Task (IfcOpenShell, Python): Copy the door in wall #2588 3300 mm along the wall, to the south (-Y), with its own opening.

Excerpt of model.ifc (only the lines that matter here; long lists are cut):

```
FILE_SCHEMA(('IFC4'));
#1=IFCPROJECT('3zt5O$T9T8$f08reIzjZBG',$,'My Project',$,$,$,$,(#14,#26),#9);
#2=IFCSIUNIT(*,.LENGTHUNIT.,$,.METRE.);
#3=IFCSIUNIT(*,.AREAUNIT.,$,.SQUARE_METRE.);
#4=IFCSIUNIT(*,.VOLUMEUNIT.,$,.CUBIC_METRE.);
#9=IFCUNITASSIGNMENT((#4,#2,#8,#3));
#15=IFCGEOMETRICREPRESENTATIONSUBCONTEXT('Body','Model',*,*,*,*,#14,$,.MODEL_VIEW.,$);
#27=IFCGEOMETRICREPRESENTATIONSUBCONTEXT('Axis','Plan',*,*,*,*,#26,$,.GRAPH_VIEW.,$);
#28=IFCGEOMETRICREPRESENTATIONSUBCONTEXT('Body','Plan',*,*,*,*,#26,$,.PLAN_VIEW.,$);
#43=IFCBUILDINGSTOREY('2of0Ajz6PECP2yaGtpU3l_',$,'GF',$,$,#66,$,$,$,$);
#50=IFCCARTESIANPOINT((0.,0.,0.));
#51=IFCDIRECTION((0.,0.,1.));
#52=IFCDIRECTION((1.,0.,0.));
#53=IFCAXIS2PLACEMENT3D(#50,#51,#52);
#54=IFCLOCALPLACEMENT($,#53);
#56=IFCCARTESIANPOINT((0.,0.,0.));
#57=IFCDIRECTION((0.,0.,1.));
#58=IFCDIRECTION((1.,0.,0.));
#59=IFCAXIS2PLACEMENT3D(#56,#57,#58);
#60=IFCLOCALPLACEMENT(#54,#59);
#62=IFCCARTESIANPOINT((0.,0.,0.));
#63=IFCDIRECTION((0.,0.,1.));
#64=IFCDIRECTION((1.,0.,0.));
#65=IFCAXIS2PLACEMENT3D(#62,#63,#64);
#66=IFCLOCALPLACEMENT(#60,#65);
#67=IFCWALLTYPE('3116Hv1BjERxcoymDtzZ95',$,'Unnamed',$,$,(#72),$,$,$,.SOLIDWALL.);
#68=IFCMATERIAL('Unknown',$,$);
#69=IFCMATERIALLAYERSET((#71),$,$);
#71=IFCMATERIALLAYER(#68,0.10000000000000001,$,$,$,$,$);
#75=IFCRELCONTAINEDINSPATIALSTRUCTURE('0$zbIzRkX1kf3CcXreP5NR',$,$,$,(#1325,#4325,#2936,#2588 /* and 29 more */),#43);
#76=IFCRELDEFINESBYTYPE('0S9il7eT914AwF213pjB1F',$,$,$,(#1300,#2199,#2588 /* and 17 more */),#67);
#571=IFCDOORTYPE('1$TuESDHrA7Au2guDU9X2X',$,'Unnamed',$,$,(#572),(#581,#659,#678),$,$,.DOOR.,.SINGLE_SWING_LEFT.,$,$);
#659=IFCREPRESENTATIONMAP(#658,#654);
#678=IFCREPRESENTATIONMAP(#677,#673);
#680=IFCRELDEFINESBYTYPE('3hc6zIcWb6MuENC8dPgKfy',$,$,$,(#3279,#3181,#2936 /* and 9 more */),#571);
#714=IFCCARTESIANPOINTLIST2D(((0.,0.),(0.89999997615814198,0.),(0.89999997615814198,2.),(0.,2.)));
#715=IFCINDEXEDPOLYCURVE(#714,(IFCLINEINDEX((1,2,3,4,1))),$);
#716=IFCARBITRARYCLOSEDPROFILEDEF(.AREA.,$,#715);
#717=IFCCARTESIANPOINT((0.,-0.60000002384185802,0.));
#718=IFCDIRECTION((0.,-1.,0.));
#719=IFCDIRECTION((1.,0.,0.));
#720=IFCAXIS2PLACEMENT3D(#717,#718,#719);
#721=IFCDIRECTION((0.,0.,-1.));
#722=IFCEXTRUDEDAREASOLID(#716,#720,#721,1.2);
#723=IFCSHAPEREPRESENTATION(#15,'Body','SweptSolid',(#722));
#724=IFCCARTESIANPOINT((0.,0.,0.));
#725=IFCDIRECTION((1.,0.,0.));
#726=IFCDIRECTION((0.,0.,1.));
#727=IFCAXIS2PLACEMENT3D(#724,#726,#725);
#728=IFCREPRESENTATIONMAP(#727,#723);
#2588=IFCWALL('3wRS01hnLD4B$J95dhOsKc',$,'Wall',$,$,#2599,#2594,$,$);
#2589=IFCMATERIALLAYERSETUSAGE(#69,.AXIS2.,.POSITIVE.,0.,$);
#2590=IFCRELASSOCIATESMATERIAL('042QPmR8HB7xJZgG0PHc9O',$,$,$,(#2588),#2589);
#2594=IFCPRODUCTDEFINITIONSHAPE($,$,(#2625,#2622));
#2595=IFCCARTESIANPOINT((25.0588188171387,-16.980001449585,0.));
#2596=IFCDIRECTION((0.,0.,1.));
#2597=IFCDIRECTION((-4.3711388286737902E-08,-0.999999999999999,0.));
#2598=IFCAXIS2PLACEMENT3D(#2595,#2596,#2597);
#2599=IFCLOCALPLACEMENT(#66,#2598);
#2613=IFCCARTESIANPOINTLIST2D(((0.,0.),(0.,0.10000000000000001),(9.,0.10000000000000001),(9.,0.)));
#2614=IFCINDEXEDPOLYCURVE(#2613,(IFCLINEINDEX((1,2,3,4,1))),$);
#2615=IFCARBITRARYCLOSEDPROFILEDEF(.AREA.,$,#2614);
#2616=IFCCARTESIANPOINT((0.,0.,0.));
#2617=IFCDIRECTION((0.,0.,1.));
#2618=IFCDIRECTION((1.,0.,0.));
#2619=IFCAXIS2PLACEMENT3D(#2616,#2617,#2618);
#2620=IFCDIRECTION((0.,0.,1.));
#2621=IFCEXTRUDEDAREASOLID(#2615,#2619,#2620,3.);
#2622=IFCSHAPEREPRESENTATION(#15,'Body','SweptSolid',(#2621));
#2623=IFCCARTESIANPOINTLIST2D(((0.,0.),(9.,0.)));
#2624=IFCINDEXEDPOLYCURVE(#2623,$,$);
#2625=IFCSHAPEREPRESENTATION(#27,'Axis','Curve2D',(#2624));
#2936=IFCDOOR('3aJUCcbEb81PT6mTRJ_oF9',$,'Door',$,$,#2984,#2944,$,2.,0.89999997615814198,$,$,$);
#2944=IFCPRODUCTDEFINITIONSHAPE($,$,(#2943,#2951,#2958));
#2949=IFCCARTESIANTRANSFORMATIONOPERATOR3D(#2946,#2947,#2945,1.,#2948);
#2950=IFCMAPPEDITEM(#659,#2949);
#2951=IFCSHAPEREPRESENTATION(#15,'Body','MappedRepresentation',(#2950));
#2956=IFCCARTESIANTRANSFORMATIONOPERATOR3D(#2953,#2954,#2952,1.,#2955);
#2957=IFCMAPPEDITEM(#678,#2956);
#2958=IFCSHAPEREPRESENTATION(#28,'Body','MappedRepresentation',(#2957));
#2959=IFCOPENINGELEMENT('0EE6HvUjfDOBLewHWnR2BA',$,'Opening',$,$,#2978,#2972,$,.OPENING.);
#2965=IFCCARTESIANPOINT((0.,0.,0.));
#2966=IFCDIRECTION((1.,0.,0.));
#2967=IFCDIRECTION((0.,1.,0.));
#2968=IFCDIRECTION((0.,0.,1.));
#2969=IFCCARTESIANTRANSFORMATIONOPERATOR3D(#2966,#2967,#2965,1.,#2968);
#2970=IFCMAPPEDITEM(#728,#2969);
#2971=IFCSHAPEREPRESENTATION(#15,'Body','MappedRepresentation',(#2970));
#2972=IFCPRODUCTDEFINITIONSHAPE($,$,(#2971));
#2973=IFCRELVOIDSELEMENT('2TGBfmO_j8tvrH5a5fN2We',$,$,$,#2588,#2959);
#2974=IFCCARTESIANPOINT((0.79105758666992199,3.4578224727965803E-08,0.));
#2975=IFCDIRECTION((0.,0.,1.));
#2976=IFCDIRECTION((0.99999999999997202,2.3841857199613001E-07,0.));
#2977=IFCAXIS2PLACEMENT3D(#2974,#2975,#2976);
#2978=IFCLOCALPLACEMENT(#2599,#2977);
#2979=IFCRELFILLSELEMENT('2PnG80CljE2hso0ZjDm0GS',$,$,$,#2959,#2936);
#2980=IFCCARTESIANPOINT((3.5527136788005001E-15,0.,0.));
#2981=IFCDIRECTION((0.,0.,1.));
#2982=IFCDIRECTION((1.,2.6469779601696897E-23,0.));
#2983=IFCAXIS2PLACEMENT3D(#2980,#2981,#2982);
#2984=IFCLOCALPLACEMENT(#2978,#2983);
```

```python
import ifcopenshell
import ifcopenshell.api.feature
import ifcopenshell.api.geometry
import ifcopenshell.api.root
import ifcopenshell.geom
import ifcopenshell.util.element
import ifcopenshell.util.placement
import ifcopenshell.util.shape
import ifcopenshell.util.unit

model = ifcopenshell.open("model.ifc")
unit_scale = ifcopenshell.util.unit.calculate_unit_scale(model)
settings = ifcopenshell.geom.settings()


def volume(element):
    """Net volume in cubic metres, openings subtracted."""
    shape = ifcopenshell.geom.create_shape(settings, element)
    return ifcopenshell.util.shape.get_volume(shape.geometry)


door = model.by_guid("3aJUCcbEb81PT6mTRJ_oF9")
opening = door.FillsVoids[0].RelatingOpeningElement
wall = opening.VoidsElements[0].RelatingBuildingElement
before = volume(wall)
shift = ifcopenshell.util.placement.get_local_placement(wall.ObjectPlacement)[:3, 0] * 3.3 / unit_scale

# copy_class copies the void relationship, type, container and properties, but no geometry.
new_opening = ifcopenshell.api.root.copy_class(model, product=opening)
new_opening.Representation = ifcopenshell.util.element.copy_deep(
    model, opening.Representation, exclude=["IfcGeometricRepresentationContext", "IfcRepresentationMap"]
)
new_door = ifcopenshell.api.root.copy_class(model, product=door)
new_door.Representation = ifcopenshell.util.element.copy_deep(
    model, door.Representation, exclude=["IfcGeometricRepresentationContext", "IfcRepresentationMap"]
)
ifcopenshell.api.feature.add_filling(model, opening=new_opening, element=new_door)

for old, new in ((opening, new_opening), (door, new_door)):
    matrix = ifcopenshell.util.placement.get_local_placement(old.ObjectPlacement)
    matrix[:3, 3] += shift
    ifcopenshell.api.geometry.edit_object_placement(model, product=new, matrix=matrix, is_si=False)

after = volume(wall)

print(f"wall volume {before:.3f} -> {after:.3f} m3")

model.write("model_updated.ifc")
```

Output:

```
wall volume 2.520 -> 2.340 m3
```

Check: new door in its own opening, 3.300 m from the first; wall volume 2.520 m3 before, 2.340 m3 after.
